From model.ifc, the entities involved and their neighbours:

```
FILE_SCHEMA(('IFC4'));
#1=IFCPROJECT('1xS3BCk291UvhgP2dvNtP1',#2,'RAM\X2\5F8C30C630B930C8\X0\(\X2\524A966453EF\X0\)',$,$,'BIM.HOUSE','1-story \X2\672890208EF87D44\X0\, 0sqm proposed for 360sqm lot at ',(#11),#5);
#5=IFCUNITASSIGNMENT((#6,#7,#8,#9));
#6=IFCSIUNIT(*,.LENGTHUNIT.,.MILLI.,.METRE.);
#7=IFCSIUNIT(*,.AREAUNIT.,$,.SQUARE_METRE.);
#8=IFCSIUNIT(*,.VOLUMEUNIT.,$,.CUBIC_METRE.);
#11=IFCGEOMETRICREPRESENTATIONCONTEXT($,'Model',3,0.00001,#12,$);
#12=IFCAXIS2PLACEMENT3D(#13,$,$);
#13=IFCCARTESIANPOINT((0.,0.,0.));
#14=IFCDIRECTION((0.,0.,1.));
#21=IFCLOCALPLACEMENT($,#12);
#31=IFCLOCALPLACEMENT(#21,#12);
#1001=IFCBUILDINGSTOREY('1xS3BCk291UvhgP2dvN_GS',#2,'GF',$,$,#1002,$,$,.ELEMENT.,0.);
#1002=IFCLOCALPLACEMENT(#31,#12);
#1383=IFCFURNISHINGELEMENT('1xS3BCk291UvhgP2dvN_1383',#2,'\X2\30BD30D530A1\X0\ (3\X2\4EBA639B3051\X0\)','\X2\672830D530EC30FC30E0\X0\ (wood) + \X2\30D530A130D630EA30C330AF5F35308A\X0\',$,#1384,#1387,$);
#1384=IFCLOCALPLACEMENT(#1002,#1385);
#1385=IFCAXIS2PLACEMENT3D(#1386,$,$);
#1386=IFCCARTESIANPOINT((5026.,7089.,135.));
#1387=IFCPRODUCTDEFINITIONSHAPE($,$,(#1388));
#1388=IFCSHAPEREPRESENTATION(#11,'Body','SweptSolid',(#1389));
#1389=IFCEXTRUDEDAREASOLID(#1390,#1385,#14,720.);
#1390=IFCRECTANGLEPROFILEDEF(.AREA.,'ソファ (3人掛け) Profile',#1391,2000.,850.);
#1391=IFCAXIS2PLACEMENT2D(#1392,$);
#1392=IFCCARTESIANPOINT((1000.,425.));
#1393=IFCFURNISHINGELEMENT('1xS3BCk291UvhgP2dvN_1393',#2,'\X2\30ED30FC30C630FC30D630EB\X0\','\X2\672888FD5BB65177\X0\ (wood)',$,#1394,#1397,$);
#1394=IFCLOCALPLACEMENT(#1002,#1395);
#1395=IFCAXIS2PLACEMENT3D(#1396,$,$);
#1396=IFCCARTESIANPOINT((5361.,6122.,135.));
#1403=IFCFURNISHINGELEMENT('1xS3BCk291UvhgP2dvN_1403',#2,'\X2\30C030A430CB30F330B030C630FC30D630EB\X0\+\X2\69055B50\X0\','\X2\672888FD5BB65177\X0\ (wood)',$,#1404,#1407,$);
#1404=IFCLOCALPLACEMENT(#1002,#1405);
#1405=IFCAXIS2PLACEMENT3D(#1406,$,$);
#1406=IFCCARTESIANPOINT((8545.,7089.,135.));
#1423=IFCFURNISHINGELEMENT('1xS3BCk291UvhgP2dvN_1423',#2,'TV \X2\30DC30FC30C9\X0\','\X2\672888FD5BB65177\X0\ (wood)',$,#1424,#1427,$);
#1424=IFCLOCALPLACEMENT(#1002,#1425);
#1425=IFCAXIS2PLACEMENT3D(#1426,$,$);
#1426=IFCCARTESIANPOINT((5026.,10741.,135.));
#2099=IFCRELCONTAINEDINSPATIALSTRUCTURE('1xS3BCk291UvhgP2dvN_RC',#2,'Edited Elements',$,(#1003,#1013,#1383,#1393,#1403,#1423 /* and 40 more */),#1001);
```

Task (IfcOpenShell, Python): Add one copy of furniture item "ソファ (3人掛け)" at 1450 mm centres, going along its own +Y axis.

```python
import ifcopenshell
import ifcopenshell.api.geometry
import ifcopenshell.api.root
import ifcopenshell.util.element
import ifcopenshell.util.placement
import ifcopenshell.util.unit

model = ifcopenshell.open("model.ifc")
unit_scale = ifcopenshell.util.unit.calculate_unit_scale(model)


def reuse_history(source, copy):
    """copy_class also copies each property set's owner history, people and application; keep the originals."""
    for rel in copy.IsDefinedBy:
        if rel.is_a("IfcRelDefinesByProperties") and (history := rel.RelatingPropertyDefinition.OwnerHistory):
            rel.RelatingPropertyDefinition.OwnerHistory = source.OwnerHistory
            ifcopenshell.util.element.remove_deep2(model, history)


source = model.by_guid("1xS3BCk291UvhgP2dvN_1383")
base = ifcopenshell.util.placement.get_local_placement(source.ObjectPlacement)
step = base[:3, 1] * 1.45 / unit_scale

for i in range(1, 2):
    copy = ifcopenshell.api.root.copy_class(model, product=source)
    copy.Representation = ifcopenshell.util.element.copy_deep(
        model, source.Representation, exclude=["IfcGeometricRepresentationContext", "IfcRepresentationMap"]
    )
    reuse_history(source, copy)
    matrix = base.copy()
    matrix[:3, 3] += i * step
    print("added at", matrix[:3, 3].round(3) + 0.0)
    ifcopenshell.api.geometry.edit_object_placement(model, product=copy, matrix=matrix, is_si=False)

model.write("model_rev.ifc")
```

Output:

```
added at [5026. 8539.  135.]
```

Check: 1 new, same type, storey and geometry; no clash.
